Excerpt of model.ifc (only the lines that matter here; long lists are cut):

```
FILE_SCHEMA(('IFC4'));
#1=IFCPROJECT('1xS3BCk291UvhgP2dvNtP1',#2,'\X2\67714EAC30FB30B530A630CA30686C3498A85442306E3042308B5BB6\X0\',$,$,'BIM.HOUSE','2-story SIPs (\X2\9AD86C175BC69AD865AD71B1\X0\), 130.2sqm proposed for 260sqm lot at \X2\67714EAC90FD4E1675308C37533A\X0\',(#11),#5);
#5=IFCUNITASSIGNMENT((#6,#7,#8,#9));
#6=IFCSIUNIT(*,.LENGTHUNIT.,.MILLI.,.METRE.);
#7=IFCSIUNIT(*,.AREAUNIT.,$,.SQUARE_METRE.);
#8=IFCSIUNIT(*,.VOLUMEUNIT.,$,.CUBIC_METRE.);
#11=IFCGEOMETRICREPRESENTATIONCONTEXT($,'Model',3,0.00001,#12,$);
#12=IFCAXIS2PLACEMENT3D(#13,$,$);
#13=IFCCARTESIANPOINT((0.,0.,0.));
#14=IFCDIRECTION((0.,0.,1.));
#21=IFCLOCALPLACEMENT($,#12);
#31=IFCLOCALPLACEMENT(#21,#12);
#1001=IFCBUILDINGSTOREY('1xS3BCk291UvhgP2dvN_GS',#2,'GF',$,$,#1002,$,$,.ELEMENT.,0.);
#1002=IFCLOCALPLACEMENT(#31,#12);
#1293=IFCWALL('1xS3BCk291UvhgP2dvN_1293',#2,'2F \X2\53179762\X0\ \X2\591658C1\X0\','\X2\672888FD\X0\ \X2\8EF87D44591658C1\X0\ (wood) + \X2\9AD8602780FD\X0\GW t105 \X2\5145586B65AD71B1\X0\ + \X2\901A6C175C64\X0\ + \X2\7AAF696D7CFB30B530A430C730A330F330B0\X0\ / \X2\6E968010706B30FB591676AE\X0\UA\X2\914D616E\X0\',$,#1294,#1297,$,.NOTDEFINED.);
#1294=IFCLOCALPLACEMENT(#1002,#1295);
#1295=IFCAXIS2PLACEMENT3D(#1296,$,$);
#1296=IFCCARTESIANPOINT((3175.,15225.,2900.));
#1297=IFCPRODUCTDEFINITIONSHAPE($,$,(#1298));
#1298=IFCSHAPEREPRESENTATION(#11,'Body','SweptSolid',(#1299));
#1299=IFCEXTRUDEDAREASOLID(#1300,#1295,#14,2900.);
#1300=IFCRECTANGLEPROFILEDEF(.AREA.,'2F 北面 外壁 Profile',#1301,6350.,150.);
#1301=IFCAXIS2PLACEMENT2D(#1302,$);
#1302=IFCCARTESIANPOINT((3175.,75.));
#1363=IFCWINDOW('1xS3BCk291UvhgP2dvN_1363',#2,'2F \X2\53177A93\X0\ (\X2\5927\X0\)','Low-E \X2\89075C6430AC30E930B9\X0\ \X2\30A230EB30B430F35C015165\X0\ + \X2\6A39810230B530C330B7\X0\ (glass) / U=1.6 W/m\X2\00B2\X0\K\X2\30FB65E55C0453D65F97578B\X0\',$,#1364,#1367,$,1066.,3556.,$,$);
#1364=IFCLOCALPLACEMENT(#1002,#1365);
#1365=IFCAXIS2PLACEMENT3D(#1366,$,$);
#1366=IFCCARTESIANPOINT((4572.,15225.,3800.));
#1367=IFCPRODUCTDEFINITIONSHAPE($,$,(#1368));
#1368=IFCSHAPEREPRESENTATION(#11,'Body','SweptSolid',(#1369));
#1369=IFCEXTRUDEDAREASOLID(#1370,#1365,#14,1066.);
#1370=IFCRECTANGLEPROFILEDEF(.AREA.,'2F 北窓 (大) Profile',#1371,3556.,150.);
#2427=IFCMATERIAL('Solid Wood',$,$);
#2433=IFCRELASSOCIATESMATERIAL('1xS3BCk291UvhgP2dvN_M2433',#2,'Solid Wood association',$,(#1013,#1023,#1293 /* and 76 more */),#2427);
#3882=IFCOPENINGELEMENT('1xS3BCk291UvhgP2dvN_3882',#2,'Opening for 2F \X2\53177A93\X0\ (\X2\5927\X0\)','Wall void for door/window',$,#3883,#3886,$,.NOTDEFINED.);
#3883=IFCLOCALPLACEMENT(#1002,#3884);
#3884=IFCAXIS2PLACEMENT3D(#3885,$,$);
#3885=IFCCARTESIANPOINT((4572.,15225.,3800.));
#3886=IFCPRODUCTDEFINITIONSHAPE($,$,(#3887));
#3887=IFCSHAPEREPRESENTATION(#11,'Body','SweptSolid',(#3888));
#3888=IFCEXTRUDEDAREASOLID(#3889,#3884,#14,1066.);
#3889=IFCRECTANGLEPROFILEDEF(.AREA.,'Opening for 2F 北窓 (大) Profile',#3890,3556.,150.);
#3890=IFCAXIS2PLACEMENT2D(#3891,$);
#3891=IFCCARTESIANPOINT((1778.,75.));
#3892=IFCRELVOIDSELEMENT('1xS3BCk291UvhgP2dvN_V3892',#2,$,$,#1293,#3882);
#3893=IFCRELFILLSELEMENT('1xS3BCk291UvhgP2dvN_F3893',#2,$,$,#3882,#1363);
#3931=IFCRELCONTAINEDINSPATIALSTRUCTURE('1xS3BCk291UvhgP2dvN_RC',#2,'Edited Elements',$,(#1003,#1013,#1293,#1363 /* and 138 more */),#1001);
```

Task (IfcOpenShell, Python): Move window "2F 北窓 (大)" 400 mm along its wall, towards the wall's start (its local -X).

```python
import ifcopenshell
import ifcopenshell.api.geometry
import ifcopenshell.util.placement
import ifcopenshell.util.unit

model = ifcopenshell.open("model.ifc")
unit_scale = ifcopenshell.util.unit.calculate_unit_scale(model)

window = model.by_id(1363)
opening = window.FillsVoids[0].RelatingOpeningElement
wall = opening.VoidsElements[0].RelatingBuildingElement

wall_matrix = ifcopenshell.util.placement.get_local_placement(wall.ObjectPlacement)
shift = wall_matrix[:3, 0] * -0.4 / unit_scale
before = ifcopenshell.util.placement.get_local_placement(window.ObjectPlacement)[:3, 3].copy()

# The window is not placed relative to its opening, so move both.
for product in (opening, window):
    matrix = ifcopenshell.util.placement.get_local_placement(product.ObjectPlacement)
    matrix[:3, 3] += shift
    ifcopenshell.api.geometry.edit_object_placement(model, product=product, matrix=matrix, is_si=False)

after = ifcopenshell.util.placement.get_local_placement(window.ObjectPlacement)[:3, 3]
print("window moved by", (after - before).round(3) + 0.0)

model.write("model_rev.ifc")
```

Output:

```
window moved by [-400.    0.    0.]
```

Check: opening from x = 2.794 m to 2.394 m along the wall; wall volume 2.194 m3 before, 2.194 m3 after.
